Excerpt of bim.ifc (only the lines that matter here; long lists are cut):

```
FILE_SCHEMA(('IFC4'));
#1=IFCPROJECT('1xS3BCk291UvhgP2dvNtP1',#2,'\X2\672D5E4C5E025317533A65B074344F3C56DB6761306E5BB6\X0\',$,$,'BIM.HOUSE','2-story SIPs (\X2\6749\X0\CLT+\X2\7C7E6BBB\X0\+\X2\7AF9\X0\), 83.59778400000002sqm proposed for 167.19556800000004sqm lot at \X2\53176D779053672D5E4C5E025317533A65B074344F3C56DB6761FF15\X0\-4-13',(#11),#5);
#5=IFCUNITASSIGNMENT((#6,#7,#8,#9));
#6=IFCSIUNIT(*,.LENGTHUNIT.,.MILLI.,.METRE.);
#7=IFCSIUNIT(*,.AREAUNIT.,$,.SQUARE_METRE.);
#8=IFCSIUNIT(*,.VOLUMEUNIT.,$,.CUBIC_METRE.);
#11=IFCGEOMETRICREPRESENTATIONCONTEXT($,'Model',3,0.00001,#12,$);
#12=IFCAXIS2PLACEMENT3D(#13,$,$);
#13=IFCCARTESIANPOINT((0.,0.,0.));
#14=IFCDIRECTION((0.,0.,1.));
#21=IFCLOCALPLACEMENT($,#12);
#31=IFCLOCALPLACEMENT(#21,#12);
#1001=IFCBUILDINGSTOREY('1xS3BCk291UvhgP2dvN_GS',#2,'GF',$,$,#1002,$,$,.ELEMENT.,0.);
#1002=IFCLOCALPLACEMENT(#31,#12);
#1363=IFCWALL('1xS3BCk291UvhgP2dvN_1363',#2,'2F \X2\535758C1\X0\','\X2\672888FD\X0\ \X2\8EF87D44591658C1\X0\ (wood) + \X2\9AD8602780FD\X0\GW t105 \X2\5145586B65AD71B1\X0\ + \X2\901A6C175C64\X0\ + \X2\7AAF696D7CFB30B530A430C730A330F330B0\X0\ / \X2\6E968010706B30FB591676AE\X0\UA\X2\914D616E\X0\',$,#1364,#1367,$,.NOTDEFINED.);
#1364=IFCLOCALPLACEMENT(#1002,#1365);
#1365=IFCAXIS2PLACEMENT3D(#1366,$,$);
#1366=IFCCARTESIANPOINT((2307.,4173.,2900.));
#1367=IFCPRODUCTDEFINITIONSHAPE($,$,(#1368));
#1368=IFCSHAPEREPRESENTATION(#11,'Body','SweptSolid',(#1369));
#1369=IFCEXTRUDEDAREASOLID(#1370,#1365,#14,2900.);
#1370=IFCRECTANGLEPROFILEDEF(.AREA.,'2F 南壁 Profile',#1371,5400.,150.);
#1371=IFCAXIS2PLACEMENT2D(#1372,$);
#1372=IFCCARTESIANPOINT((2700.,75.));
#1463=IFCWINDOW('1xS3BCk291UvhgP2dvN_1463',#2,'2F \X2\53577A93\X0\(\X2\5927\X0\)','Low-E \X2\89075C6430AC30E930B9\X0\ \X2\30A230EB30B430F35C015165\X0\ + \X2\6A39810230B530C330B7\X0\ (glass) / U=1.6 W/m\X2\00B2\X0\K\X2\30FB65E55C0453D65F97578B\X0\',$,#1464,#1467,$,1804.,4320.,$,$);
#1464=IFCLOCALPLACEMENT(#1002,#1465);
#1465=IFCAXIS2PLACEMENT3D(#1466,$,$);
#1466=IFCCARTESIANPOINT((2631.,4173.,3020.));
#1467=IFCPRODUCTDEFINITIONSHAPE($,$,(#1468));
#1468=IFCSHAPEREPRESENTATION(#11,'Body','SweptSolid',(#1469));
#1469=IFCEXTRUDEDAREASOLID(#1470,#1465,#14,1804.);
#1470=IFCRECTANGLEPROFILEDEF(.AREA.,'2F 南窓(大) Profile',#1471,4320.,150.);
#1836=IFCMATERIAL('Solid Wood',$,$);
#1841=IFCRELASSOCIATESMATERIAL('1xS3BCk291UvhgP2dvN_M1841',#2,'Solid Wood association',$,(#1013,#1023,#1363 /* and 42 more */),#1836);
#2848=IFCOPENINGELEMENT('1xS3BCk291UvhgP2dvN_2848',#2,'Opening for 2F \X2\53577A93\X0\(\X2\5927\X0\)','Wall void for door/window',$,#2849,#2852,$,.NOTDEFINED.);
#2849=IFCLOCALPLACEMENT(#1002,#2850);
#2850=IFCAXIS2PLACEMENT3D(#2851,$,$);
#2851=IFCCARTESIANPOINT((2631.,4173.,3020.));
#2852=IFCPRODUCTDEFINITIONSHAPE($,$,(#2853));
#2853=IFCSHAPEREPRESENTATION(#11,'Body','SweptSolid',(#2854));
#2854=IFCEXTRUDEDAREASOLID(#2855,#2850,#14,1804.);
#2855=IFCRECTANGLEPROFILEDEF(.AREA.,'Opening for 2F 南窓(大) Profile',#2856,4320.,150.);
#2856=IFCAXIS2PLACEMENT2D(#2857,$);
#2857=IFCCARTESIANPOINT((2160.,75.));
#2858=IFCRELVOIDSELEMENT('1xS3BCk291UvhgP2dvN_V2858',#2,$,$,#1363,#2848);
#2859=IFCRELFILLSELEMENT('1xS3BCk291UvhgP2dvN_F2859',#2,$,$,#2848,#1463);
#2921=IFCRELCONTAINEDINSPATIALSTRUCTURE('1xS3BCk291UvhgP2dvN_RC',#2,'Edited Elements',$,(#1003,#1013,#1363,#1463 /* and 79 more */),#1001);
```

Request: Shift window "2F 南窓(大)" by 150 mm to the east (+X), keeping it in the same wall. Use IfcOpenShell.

```python
import ifcopenshell
import ifcopenshell.api.geometry
import ifcopenshell.util.placement

model = ifcopenshell.open("bim.ifc")

window = model.by_id(1463)
opening = window.FillsVoids[0].RelatingOpeningElement
wall = opening.VoidsElements[0].RelatingBuildingElement

wall_matrix = ifcopenshell.util.placement.get_local_placement(wall.ObjectPlacement)
shift = wall_matrix[:3, 0] * 150.0
before = ifcopenshell.util.placement.get_local_placement(window.ObjectPlacement)[:3, 3].copy()

# The window is not placed relative to its opening, so move both.
for product in (opening, window):
    matrix = ifcopenshell.util.placement.get_local_placement(product.ObjectPlacement)
    matrix[:3, 3] += shift
    ifcopenshell.api.geometry.edit_object_placement(model, product=product, matrix=matrix, is_si=False)

after = ifcopenshell.util.placement.get_local_placement(window.ObjectPlacement)[:3, 3]
print("window moved by", (after - before).round(3) + 0.0)

model.write("bim_v2.ifc")
```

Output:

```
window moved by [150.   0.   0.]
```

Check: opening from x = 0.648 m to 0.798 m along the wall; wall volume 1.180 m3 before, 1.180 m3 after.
